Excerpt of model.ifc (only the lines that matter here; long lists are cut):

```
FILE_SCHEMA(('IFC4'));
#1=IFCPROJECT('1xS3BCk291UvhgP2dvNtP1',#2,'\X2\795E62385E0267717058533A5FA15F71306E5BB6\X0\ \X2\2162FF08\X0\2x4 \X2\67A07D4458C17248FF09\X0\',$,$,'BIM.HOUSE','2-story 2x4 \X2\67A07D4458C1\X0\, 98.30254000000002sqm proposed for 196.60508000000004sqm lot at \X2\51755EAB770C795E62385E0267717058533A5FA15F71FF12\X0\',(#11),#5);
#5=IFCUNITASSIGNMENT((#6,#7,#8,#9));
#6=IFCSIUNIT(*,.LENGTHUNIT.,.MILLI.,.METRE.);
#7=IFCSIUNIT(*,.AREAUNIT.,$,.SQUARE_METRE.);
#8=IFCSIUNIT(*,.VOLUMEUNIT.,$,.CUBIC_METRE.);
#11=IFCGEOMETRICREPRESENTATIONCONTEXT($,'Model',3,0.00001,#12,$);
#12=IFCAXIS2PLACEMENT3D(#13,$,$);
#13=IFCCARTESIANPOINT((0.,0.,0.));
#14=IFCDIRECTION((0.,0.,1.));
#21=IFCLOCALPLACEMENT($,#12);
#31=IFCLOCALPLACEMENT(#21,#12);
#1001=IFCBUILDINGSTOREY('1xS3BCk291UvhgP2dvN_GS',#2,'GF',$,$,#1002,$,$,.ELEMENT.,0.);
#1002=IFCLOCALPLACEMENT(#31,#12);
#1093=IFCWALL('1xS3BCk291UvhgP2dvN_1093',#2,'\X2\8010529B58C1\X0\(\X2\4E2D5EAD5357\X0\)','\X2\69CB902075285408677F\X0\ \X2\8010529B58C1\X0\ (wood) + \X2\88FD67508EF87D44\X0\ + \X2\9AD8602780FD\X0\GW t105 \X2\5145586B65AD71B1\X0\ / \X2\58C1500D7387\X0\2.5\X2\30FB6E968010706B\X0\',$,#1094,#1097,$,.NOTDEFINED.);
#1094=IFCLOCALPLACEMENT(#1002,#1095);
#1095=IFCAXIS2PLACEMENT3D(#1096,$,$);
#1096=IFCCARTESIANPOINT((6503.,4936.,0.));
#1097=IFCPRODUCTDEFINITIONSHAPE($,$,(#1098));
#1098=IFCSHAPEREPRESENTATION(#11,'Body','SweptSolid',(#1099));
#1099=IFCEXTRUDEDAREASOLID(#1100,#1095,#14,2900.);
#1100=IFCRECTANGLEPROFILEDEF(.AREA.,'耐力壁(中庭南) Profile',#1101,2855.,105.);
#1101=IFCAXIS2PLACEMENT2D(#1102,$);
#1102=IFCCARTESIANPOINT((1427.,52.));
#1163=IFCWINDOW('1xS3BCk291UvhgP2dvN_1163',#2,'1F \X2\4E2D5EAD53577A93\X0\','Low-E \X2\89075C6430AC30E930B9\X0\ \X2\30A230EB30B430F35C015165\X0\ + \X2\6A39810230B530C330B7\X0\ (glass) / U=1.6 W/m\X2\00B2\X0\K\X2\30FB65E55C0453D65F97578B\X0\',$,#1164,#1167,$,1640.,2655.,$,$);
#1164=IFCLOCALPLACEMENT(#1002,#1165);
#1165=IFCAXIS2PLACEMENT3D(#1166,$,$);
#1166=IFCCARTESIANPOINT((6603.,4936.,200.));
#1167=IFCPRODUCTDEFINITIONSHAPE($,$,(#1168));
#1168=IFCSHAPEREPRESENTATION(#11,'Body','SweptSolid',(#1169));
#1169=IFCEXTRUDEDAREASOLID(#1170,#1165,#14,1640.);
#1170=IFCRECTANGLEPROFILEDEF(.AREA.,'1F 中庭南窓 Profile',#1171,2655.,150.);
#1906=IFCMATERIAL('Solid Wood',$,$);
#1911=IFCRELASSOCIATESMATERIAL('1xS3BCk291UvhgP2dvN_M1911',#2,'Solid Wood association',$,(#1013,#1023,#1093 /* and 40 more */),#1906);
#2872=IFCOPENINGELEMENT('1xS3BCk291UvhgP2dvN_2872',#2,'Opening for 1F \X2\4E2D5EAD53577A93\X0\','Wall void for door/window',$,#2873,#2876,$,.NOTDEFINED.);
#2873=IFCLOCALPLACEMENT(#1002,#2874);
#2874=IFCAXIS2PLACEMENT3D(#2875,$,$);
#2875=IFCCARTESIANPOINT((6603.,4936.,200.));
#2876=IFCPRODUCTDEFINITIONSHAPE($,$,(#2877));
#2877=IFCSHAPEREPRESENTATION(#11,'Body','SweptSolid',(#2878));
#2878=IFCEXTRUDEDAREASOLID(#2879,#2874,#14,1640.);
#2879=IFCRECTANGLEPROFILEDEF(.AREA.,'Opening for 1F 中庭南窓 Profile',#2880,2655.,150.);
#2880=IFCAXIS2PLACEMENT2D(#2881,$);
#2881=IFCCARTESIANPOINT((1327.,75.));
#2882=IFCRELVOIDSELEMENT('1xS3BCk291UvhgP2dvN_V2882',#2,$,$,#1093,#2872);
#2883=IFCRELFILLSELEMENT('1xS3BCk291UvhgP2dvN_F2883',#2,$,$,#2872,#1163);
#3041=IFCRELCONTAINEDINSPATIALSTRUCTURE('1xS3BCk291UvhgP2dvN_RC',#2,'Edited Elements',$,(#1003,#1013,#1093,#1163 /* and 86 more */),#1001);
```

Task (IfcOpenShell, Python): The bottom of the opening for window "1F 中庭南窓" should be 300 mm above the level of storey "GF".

```python
import numpy as np
import ifcopenshell
import ifcopenshell.api.geometry
import ifcopenshell.geom
import ifcopenshell.util.element
import ifcopenshell.util.placement
import ifcopenshell.util.shape
import ifcopenshell.util.unit

model = ifcopenshell.open("model.ifc")
unit_scale = ifcopenshell.util.unit.calculate_unit_scale(model)

window = model.by_id(1163)
opening = window.FillsVoids[0].RelatingOpeningElement
storey = ifcopenshell.util.element.get_container(window, ifc_class="IfcBuildingStorey")
level = ifcopenshell.util.placement.get_local_placement(storey.ObjectPlacement)[2, 3]

# The opening's origin need not be at the sill, so measure its lowest point.
shape = ifcopenshell.geom.create_shape(ifcopenshell.geom.settings(), opening)
bottom = ifcopenshell.util.shape.get_shape_bottom_elevation(shape, shape.geometry) / unit_scale
dz = level + 300.0 - bottom

shift = np.array([0.0, 0.0, dz])
# The window is not placed relative to its opening, so move both.
for product in (opening, window):
    matrix = ifcopenshell.util.placement.get_local_placement(product.ObjectPlacement)
    matrix[:3, 3] += shift
    ifcopenshell.api.geometry.edit_object_placement(model, product=product, matrix=matrix, is_si=False)

print(f"moved by {dz * unit_scale:+.3f} m")

model.write("model_updated.ifc")
```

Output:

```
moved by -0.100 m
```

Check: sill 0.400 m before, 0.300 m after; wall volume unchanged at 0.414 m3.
